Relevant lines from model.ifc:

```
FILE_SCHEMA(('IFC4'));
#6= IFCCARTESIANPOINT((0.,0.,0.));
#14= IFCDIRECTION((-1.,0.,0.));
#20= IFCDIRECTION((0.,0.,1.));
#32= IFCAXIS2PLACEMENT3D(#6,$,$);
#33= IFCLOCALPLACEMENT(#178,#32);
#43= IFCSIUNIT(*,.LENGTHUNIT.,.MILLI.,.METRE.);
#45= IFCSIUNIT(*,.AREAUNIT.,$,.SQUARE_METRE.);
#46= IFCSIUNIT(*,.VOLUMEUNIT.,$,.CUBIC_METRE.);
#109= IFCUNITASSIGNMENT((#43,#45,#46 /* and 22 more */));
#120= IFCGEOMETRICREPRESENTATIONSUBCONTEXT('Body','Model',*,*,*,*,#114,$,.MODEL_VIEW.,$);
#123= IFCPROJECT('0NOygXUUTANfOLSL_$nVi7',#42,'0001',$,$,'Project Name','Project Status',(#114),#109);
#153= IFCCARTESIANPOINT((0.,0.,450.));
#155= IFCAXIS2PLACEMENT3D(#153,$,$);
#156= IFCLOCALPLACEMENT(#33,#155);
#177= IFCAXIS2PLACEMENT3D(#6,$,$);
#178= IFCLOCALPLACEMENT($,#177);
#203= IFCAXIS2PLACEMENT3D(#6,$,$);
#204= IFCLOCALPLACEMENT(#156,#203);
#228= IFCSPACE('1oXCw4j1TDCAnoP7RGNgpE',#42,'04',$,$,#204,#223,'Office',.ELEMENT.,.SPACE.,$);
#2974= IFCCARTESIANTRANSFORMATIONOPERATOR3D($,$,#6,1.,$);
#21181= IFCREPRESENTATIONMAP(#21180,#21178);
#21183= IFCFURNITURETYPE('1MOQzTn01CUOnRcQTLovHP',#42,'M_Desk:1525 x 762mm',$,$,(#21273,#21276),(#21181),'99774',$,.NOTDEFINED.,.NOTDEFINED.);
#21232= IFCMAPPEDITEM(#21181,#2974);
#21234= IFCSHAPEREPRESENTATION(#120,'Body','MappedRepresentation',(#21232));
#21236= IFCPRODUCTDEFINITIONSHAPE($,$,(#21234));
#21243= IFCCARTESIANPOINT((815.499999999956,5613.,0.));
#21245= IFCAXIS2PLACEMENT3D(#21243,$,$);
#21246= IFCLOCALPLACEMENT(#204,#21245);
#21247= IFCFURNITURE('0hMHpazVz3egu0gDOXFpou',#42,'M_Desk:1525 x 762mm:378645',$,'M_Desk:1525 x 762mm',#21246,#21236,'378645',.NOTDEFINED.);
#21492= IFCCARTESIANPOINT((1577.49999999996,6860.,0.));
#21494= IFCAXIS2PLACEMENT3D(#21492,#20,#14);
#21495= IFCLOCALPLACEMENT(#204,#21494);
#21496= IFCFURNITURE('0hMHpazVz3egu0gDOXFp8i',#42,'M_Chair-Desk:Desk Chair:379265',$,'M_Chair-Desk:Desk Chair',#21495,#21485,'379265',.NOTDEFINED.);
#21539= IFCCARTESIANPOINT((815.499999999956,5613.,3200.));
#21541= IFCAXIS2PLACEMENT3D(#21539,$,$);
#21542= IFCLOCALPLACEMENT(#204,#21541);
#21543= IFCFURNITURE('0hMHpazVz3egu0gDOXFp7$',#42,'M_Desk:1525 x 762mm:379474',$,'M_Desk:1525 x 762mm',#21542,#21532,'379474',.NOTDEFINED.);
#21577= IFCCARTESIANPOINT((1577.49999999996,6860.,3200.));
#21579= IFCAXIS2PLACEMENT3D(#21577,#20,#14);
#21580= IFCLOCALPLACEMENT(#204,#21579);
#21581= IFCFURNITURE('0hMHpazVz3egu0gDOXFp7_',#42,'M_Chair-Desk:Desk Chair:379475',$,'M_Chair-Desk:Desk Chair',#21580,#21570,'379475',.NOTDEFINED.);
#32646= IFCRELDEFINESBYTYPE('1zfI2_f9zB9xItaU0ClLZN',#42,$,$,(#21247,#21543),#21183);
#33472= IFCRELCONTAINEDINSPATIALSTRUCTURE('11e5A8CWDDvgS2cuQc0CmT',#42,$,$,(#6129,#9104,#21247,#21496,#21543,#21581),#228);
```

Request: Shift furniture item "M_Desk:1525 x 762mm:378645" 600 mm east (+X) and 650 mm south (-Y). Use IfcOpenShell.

```python
import ifcopenshell
import ifcopenshell.api.geometry
import ifcopenshell.util.placement
import ifcopenshell.util.unit

model = ifcopenshell.open("model.ifc")
unit_scale = ifcopenshell.util.unit.calculate_unit_scale(model)

item = model.by_id(21247)
matrix = ifcopenshell.util.placement.get_local_placement(item.ObjectPlacement)
matrix[0, 3] += 0.6 / unit_scale
matrix[1, 3] -= 0.65 / unit_scale
ifcopenshell.api.geometry.edit_object_placement(model, product=item, matrix=matrix, is_si=False)

print(ifcopenshell.util.placement.get_local_placement(item.ObjectPlacement).round(3) + 0.0)

model.write("model-out.ifc")
```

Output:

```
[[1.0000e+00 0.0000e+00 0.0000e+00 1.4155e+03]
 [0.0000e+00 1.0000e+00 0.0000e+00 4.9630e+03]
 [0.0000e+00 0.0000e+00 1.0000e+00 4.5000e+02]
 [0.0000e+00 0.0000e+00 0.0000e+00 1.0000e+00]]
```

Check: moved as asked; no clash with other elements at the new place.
